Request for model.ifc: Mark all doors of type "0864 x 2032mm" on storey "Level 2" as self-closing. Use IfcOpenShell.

First a look at what the model holds.

```python
import ifcopenshell
import ifcopenshell.util.element

model = ifcopenshell.open("model.ifc")
print(model.schema)
storey = next(s for s in model.by_type("IfcBuildingStorey") if s.Name == "Level 2")
doors = [e for e in ifcopenshell.util.element.get_decomposition(storey) if e.is_a("IfcDoor")]
seen = {}
for e in doors:
    element_type = ifcopenshell.util.element.get_type(e)
    key = (element_type.Name if element_type != e and element_type else None, ifcopenshell.util.element.get_pset(e, "Pset_DoorCommon", "SelfClosing"))
    seen[key] = seen.get(key, 0) + 1
for (name, value), count in sorted(seen.items(), key=str):
    print(count, "x", name, "|", value)
```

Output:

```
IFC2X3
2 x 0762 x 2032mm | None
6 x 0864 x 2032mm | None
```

```python
import ifcopenshell
import ifcopenshell.api.pset
import ifcopenshell.util.element

model = ifcopenshell.open("model.ifc")

storey = next(s for s in model.by_type("IfcBuildingStorey") if s.Name == "Level 2")
doors = [e for e in ifcopenshell.util.element.get_decomposition(storey) if e.is_a("IfcDoor")]

count = 0
for e in doors:
    element_type = ifcopenshell.util.element.get_type(e)
    if element_type in (None, e) or element_type.Name != "0864 x 2032mm":
        continue
    # add_pset returns the element's existing set when there is one.
    pset = ifcopenshell.api.pset.add_pset(model, product=e, name="Pset_DoorCommon")
    ifcopenshell.api.pset.edit_pset(model, pset=pset, properties={"SelfClosing": True})
    count += 1

print(count, "doors updated")

model.write("model_updated.ifc")
```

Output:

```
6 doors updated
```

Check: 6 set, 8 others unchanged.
